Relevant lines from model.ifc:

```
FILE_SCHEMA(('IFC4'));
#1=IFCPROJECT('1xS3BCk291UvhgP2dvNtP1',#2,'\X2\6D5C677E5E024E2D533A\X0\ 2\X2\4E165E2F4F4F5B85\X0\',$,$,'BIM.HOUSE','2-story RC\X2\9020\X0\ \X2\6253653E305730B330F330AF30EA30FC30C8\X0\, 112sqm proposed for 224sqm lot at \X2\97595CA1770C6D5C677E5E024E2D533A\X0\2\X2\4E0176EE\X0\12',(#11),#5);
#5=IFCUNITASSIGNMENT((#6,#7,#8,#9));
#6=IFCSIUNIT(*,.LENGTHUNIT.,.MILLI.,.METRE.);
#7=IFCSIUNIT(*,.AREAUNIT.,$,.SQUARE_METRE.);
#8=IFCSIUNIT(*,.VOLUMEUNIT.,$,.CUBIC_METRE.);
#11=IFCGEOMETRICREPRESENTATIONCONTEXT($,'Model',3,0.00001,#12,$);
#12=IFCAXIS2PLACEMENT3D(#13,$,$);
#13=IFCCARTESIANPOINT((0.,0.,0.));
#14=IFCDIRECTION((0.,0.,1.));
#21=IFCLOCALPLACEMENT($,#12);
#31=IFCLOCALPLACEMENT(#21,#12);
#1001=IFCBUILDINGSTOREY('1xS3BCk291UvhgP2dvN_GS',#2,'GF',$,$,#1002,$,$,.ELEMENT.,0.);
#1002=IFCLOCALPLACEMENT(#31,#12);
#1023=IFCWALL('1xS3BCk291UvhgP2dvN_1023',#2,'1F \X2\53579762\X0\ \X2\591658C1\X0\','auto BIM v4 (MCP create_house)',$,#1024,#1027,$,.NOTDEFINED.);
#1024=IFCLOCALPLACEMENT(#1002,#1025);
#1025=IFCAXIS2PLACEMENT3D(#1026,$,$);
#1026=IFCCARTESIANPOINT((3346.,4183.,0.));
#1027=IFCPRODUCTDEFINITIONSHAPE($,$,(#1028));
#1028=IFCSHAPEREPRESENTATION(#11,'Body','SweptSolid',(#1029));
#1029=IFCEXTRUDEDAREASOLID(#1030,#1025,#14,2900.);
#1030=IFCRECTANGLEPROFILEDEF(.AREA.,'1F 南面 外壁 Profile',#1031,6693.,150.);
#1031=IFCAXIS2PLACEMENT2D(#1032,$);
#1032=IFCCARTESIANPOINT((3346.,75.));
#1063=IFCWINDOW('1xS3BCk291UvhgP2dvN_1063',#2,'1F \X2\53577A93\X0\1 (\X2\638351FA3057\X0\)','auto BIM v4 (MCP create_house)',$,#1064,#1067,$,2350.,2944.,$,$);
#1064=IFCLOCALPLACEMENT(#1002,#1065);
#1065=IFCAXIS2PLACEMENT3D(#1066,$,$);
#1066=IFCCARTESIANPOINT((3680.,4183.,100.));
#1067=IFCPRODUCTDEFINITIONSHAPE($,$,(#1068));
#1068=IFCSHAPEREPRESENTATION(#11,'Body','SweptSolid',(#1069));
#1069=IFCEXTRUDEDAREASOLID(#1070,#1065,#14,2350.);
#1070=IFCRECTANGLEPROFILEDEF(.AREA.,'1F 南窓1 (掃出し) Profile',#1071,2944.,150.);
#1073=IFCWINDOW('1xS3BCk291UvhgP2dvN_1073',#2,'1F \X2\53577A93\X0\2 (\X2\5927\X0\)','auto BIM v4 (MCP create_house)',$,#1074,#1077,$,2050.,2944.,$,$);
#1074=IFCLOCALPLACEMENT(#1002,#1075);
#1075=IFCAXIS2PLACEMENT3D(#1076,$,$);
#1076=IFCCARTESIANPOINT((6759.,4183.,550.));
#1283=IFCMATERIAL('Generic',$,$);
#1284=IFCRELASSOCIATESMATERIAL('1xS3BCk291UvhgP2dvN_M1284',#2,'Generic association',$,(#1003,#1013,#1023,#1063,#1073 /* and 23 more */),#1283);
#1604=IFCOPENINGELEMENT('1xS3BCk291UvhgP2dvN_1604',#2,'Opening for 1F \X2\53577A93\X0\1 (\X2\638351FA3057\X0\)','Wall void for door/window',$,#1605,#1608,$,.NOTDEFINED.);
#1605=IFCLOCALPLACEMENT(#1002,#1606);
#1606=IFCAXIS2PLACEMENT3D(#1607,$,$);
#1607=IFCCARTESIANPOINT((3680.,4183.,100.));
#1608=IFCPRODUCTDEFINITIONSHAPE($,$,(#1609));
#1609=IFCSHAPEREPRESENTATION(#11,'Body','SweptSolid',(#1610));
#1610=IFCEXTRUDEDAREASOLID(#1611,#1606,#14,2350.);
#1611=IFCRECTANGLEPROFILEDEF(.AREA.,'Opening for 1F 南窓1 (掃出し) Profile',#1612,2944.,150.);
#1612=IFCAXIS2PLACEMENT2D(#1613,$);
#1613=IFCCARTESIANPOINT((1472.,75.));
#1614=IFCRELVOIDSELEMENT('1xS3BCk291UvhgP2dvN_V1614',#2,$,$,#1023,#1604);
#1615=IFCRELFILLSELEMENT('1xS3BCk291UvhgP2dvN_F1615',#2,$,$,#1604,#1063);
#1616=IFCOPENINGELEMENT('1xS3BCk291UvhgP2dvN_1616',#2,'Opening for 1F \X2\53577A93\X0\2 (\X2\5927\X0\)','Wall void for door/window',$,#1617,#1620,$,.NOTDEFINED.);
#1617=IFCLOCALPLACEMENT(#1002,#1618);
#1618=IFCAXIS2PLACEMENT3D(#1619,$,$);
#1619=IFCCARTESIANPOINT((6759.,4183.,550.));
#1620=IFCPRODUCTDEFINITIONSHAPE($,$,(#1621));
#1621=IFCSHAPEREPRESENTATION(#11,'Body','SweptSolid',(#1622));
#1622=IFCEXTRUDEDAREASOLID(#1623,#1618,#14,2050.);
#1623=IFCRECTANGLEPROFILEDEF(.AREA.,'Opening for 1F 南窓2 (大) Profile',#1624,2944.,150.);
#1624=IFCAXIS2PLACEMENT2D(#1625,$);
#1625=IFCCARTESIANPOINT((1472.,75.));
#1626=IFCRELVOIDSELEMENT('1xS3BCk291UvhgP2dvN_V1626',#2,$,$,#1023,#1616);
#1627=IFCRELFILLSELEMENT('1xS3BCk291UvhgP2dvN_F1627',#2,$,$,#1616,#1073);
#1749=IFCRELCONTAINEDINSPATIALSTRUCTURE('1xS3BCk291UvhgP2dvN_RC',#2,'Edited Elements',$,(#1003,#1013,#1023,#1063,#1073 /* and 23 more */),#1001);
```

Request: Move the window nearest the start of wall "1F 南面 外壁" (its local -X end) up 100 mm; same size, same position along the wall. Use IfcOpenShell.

```python
import numpy as np
import ifcopenshell
import ifcopenshell.api.geometry
import ifcopenshell.util.placement
import ifcopenshell.util.unit

model = ifcopenshell.open("model.ifc")
unit_scale = ifcopenshell.util.unit.calculate_unit_scale(model)

window = model.by_guid("1xS3BCk291UvhgP2dvN_1063")
opening = window.FillsVoids[0].RelatingOpeningElement
dz = 100.0

shift = np.array([0.0, 0.0, dz])
# The window is not placed relative to its opening, so move both.
for product in (opening, window):
    matrix = ifcopenshell.util.placement.get_local_placement(product.ObjectPlacement)
    matrix[:3, 3] += shift
    ifcopenshell.api.geometry.edit_object_placement(model, product=product, matrix=matrix, is_si=False)

print(f"moved by {dz * unit_scale:+.3f} m")

model.write("model_rev.ifc")
```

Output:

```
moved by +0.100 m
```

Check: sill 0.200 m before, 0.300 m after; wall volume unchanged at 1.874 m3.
